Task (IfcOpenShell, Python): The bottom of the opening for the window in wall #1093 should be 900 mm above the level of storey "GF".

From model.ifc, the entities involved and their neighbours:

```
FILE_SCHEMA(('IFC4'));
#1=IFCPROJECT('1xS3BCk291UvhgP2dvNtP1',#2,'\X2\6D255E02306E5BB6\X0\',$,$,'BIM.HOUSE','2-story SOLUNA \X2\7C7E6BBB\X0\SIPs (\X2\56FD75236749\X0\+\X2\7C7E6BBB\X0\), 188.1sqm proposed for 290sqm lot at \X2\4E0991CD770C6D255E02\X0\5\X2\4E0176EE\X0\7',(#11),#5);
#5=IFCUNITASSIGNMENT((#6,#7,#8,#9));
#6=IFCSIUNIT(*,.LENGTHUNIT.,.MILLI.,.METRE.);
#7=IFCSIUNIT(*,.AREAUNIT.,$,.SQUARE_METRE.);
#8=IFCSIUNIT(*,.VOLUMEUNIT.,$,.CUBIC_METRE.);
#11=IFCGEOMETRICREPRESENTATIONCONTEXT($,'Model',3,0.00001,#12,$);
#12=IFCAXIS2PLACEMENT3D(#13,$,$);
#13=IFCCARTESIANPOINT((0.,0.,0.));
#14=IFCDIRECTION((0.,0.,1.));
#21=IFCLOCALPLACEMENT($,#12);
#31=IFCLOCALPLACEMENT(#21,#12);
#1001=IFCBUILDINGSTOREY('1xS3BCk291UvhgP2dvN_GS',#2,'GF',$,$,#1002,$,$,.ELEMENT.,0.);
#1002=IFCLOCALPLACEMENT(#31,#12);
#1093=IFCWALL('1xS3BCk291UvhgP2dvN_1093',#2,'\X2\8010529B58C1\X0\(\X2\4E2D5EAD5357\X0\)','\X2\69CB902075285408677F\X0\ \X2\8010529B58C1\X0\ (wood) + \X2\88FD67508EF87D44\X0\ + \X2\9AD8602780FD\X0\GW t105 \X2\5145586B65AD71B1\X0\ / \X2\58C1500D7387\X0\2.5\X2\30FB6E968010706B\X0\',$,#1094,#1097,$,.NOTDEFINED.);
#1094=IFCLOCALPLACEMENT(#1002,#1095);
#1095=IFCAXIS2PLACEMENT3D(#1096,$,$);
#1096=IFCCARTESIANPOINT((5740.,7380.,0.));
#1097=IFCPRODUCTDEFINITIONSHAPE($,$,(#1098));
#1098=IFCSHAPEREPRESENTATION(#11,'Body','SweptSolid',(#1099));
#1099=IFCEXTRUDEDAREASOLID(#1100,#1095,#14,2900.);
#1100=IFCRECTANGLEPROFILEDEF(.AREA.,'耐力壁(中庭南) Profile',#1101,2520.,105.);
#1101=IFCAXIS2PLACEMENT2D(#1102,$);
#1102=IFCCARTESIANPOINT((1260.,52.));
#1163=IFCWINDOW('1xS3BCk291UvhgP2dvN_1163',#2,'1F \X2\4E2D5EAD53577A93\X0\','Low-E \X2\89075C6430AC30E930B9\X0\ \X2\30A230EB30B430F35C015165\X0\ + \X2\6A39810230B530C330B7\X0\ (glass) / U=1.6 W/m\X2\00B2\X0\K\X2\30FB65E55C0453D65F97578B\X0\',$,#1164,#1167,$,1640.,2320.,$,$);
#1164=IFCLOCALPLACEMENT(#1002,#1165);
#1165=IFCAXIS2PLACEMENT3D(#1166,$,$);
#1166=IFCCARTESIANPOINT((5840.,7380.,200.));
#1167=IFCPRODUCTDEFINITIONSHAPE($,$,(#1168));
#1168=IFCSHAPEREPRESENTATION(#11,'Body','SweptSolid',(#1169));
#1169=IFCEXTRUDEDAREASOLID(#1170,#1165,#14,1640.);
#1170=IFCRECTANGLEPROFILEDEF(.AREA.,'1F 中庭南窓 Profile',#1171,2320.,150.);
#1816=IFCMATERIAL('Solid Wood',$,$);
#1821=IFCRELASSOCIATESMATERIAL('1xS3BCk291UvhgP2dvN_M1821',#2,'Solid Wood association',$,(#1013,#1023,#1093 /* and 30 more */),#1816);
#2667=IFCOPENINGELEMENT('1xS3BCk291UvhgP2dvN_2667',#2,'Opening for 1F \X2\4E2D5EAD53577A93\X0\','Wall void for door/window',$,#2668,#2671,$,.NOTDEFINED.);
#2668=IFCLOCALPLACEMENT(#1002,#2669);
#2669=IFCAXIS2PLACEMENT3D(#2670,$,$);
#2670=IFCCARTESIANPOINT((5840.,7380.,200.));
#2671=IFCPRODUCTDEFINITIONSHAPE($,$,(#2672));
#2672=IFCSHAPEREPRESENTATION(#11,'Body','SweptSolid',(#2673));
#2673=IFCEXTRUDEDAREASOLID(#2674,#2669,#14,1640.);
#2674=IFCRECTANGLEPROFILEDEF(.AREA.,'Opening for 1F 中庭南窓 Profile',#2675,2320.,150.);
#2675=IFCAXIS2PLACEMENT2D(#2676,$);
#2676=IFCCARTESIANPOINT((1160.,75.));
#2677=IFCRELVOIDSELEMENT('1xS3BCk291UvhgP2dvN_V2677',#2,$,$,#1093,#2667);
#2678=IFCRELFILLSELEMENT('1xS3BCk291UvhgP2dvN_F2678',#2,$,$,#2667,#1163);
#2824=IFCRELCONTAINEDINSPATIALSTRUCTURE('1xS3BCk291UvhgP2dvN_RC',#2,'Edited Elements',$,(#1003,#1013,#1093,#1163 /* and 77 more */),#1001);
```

```python
import numpy as np
import ifcopenshell
import ifcopenshell.api.geometry
import ifcopenshell.geom
import ifcopenshell.util.element
import ifcopenshell.util.placement
import ifcopenshell.util.shape
import ifcopenshell.util.unit

model = ifcopenshell.open("model.ifc")
unit_scale = ifcopenshell.util.unit.calculate_unit_scale(model)

window = model.by_id(1163)
opening = window.FillsVoids[0].RelatingOpeningElement
storey = ifcopenshell.util.element.get_container(window, ifc_class="IfcBuildingStorey")
level = ifcopenshell.util.placement.get_local_placement(storey.ObjectPlacement)[2, 3]

# The opening's origin need not be at the sill, so measure its lowest point.
shape = ifcopenshell.geom.create_shape(ifcopenshell.geom.settings(), opening)
bottom = ifcopenshell.util.shape.get_shape_bottom_elevation(shape, shape.geometry) / unit_scale
dz = level + 0.9 / unit_scale - bottom

shift = np.array([0.0, 0.0, dz])
# The window is not placed relative to its opening, so move both.
for product in (opening, window):
    matrix = ifcopenshell.util.placement.get_local_placement(product.ObjectPlacement)
    matrix[:3, 3] += shift
    ifcopenshell.api.geometry.edit_object_placement(model, product=product, matrix=matrix, is_si=False)

print(f"moved by {dz * unit_scale:+.3f} m")

model.write("model_edited.ifc")
```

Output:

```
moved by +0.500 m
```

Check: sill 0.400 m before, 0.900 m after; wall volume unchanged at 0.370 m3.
